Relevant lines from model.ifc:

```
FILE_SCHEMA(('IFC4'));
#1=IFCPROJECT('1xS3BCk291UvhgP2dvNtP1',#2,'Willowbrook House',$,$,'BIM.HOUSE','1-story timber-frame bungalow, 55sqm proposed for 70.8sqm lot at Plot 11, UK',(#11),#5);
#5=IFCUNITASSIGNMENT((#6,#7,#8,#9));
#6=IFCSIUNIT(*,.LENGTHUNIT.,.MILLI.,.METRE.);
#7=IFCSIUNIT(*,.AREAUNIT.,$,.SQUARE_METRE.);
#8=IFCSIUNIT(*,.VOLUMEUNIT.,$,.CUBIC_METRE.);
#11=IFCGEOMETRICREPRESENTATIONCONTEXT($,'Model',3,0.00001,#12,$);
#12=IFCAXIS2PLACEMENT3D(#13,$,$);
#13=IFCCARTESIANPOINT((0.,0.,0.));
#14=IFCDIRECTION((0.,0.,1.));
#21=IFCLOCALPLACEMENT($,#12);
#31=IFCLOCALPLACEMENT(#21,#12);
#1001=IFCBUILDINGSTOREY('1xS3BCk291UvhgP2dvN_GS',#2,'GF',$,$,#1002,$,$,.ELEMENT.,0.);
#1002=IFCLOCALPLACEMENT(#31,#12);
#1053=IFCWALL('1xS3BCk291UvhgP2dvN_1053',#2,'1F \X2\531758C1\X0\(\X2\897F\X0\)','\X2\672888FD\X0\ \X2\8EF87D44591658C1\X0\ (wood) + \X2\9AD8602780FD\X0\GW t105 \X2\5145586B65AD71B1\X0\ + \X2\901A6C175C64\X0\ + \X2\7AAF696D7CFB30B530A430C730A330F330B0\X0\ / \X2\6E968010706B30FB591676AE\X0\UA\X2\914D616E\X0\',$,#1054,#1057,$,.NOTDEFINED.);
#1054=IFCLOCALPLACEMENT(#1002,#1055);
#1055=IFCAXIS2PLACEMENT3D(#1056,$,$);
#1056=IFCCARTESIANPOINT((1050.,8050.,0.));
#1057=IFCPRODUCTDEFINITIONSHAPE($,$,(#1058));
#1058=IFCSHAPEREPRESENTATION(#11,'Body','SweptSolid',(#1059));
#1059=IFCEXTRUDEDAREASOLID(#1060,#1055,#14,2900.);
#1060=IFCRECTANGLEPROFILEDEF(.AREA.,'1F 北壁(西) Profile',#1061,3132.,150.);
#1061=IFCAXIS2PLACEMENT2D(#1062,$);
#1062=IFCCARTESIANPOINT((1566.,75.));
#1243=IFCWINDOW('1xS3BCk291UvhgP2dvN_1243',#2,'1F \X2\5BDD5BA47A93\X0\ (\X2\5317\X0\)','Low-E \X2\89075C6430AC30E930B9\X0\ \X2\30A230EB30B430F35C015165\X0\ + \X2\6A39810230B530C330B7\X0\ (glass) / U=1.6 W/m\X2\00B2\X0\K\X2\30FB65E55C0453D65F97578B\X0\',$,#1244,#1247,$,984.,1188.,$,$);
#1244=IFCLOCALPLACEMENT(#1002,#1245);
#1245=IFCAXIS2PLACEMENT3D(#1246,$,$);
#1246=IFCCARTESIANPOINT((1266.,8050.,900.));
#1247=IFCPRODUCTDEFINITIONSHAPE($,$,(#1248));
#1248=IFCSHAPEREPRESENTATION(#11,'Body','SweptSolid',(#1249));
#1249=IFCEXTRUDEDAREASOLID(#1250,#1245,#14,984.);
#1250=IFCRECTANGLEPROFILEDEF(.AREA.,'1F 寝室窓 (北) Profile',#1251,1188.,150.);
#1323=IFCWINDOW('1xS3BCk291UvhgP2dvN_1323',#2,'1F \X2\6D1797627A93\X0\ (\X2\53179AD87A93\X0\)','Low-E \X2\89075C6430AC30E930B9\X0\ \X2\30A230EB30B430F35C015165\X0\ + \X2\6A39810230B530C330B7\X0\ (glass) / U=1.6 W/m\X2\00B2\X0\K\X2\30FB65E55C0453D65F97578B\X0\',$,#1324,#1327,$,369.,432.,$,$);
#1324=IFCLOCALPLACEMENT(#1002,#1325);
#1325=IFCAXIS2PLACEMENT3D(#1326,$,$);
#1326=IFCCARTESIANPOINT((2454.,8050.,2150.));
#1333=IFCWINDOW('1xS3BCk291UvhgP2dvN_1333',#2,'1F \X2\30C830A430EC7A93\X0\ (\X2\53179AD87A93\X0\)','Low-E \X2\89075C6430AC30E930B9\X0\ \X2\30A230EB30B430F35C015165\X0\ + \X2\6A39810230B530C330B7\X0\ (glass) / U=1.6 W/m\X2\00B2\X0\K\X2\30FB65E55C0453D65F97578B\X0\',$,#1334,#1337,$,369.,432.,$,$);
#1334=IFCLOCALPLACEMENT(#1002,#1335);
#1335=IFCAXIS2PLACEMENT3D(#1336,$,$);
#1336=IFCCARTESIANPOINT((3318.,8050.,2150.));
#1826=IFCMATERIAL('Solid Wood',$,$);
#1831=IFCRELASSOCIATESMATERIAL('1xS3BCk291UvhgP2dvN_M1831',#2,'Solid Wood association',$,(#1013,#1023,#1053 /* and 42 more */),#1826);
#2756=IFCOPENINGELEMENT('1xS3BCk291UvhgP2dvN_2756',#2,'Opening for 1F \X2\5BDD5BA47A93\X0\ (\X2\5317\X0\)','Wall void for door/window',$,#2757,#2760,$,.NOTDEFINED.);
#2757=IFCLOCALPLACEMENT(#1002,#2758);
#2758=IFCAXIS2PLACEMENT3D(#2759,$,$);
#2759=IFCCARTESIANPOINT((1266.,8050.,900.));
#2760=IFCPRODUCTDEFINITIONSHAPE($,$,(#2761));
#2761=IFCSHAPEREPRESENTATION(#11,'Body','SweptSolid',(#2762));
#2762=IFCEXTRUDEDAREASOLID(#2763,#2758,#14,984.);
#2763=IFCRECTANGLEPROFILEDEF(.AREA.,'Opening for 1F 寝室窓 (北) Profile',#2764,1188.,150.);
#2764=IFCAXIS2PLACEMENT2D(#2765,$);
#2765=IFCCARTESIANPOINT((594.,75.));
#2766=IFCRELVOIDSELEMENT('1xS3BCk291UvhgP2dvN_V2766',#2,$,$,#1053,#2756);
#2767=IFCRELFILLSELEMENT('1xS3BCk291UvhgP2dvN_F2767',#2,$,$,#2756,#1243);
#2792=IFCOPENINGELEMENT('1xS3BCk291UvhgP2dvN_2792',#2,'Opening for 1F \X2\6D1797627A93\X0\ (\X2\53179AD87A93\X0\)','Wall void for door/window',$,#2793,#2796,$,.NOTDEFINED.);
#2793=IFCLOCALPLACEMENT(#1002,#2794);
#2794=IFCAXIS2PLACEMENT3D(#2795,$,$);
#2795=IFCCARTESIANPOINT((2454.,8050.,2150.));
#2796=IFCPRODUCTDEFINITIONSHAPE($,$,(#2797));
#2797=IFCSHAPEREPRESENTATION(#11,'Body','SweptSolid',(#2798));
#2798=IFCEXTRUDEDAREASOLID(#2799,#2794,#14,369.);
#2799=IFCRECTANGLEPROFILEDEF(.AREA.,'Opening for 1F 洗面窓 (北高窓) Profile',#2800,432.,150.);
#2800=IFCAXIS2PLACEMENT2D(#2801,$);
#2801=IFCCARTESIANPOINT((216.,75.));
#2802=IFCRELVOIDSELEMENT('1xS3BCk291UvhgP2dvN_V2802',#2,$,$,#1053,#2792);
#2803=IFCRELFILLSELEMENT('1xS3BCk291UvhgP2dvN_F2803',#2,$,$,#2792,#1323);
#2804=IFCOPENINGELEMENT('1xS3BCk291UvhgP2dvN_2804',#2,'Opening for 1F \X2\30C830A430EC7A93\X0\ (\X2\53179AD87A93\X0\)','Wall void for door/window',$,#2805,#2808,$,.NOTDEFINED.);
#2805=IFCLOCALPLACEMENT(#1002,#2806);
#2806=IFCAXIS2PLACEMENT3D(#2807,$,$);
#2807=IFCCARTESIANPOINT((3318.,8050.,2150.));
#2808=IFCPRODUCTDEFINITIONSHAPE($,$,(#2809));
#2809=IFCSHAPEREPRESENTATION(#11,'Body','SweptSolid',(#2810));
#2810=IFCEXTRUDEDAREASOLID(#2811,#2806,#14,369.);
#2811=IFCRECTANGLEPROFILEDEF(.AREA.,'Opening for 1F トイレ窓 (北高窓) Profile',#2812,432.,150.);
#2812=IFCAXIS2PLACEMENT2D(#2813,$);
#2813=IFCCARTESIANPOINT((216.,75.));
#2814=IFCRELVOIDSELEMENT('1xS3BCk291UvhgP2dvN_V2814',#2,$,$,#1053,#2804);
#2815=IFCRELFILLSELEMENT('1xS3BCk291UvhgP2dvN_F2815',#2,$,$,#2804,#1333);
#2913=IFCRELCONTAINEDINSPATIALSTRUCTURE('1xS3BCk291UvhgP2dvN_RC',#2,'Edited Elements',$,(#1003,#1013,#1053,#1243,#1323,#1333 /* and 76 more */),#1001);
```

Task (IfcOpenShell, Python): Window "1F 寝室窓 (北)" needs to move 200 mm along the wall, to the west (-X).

```python
import ifcopenshell
import ifcopenshell.api.geometry
import ifcopenshell.util.placement
import ifcopenshell.util.unit

model = ifcopenshell.open("model.ifc")
unit_scale = ifcopenshell.util.unit.calculate_unit_scale(model)

window = model.by_guid("1xS3BCk291UvhgP2dvN_1243")
opening = window.FillsVoids[0].RelatingOpeningElement
wall = opening.VoidsElements[0].RelatingBuildingElement

wall_matrix = ifcopenshell.util.placement.get_local_placement(wall.ObjectPlacement)
shift = wall_matrix[:3, 0] * -0.2 / unit_scale
before = ifcopenshell.util.placement.get_local_placement(window.ObjectPlacement)[:3, 3].copy()

# The window is not placed relative to its opening, so move both.
for product in (opening, window):
    matrix = ifcopenshell.util.placement.get_local_placement(product.ObjectPlacement)
    matrix[:3, 3] += shift
    ifcopenshell.api.geometry.edit_object_placement(model, product=product, matrix=matrix, is_si=False)

after = ifcopenshell.util.placement.get_local_placement(window.ObjectPlacement)[:3, 3]
print("window moved by", (after - before).round(3) + 0.0)

model.write("model_edited.ifc")
```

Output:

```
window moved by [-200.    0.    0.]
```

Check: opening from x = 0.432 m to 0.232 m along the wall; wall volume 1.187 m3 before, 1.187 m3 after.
